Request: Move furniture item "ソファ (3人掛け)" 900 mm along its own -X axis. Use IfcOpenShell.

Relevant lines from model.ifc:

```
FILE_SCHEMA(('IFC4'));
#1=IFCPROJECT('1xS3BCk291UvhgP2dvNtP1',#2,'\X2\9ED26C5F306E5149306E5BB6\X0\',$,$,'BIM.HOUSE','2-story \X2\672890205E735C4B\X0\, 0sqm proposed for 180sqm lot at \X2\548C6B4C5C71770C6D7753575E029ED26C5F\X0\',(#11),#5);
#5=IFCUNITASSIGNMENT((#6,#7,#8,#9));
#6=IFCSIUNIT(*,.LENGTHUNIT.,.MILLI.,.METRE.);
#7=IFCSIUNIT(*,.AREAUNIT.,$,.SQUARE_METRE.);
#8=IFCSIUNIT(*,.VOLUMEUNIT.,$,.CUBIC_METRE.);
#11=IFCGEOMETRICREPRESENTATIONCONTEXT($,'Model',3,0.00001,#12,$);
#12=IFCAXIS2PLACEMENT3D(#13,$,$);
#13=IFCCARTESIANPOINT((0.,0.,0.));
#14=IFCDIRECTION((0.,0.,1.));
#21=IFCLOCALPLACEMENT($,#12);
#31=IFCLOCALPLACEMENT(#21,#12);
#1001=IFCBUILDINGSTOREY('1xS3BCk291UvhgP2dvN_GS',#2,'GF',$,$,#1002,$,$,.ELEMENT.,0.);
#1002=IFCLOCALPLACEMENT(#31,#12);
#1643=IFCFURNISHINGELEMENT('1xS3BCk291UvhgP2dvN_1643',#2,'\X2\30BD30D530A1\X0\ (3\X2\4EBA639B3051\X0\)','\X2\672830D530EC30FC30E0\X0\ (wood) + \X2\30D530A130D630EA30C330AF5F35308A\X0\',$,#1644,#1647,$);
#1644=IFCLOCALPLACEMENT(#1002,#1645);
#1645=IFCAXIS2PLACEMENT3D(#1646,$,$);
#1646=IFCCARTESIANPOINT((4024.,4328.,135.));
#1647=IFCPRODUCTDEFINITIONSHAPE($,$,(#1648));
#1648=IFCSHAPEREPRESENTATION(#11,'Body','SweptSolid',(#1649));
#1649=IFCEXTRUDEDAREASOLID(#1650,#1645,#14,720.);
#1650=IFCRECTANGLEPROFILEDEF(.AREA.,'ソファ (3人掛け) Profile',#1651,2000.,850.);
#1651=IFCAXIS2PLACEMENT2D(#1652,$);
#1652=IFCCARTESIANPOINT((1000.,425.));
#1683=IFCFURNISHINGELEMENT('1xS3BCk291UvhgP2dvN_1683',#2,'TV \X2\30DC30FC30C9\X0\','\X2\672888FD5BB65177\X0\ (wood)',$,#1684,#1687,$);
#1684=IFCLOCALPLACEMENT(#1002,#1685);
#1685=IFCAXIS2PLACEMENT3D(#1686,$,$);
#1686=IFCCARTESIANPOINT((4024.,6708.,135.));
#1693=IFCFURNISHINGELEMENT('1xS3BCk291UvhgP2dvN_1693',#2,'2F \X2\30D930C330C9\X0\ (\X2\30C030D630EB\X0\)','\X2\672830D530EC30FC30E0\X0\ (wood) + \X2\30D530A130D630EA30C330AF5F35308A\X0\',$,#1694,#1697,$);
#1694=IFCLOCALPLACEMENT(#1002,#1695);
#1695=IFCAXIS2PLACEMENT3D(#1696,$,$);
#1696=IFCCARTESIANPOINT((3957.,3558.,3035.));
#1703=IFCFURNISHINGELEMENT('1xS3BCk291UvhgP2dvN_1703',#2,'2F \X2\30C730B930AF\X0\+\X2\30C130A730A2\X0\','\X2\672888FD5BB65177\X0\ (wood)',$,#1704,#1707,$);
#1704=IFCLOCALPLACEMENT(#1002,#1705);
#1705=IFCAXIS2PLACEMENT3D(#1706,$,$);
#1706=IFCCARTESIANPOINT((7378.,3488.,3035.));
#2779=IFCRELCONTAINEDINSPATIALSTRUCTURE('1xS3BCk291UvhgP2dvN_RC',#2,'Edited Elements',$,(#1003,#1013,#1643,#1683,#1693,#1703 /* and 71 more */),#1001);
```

```python
import ifcopenshell
import ifcopenshell.api.geometry
import ifcopenshell.util.placement
import ifcopenshell.util.unit

model = ifcopenshell.open("model.ifc")
unit_scale = ifcopenshell.util.unit.calculate_unit_scale(model)

item = model.by_guid("1xS3BCk291UvhgP2dvN_1643")
matrix = ifcopenshell.util.placement.get_local_placement(item.ObjectPlacement)
matrix[:3, 3] -= matrix[:3, 0] * 0.9 / unit_scale
ifcopenshell.api.geometry.edit_object_placement(model, product=item, matrix=matrix, is_si=False)

print(ifcopenshell.util.placement.get_local_placement(item.ObjectPlacement).round(3) + 0.0)

model.write("model_updated.ifc")
```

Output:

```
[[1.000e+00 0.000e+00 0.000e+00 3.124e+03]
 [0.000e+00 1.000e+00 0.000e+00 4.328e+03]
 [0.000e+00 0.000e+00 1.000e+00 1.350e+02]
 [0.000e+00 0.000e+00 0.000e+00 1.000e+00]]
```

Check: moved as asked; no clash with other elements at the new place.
